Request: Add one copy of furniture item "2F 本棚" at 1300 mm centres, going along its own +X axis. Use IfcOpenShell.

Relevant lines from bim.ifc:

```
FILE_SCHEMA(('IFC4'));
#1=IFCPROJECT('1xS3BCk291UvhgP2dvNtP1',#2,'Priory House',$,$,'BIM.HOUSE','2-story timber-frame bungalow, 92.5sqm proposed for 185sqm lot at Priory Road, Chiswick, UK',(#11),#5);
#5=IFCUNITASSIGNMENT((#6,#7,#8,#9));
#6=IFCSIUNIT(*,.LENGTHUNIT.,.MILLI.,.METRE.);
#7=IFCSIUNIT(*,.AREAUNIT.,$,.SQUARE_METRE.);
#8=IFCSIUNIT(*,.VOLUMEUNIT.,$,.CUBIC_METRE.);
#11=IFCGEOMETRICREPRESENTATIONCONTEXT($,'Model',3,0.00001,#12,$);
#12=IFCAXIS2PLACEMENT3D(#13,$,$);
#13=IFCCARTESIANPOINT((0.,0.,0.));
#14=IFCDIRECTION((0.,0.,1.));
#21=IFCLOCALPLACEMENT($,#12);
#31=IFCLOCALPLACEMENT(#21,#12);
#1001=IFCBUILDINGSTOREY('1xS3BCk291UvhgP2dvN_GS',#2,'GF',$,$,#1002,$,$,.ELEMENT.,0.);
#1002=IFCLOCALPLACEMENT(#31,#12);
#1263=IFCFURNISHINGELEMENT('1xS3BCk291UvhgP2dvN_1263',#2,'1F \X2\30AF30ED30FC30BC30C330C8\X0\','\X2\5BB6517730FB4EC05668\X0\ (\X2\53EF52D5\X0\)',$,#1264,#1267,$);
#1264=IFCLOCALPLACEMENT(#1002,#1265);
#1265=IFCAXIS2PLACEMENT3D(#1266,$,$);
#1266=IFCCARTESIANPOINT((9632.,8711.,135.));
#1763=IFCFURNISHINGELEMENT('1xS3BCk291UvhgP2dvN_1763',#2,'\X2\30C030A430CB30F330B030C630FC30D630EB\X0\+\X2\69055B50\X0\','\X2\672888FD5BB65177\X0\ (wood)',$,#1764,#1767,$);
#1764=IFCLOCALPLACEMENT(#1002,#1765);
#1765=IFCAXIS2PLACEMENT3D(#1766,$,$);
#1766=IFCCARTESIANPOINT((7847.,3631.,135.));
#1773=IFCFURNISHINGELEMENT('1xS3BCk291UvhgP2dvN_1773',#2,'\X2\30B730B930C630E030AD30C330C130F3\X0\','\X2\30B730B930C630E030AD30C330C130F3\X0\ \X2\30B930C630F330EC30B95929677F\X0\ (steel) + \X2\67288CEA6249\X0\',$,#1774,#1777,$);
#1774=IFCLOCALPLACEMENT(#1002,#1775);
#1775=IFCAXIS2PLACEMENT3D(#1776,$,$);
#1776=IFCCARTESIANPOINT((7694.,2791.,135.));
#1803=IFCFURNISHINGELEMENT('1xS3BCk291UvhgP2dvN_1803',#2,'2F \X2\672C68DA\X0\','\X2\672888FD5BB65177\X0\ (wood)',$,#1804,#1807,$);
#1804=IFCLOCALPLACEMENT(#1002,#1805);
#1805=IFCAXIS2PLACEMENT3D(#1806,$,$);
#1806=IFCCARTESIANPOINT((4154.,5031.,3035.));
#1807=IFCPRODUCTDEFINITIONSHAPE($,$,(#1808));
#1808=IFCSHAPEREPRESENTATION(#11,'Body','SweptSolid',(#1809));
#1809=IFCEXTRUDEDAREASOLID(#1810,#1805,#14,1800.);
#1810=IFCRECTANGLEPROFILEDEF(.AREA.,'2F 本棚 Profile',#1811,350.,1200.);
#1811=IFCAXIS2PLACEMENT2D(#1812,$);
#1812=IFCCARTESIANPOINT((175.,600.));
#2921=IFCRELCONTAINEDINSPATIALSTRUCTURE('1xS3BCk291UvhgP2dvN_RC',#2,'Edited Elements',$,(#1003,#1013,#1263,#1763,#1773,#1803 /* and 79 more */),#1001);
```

```python
import ifcopenshell
import ifcopenshell.api.geometry
import ifcopenshell.api.root
import ifcopenshell.util.element
import ifcopenshell.util.placement
import ifcopenshell.util.unit

model = ifcopenshell.open("bim.ifc")
unit_scale = ifcopenshell.util.unit.calculate_unit_scale(model)


def reuse_history(source, copy):
    """copy_class also copies each property set's owner history, people and application; keep the originals."""
    for rel in copy.IsDefinedBy:
        if rel.is_a("IfcRelDefinesByProperties") and (history := rel.RelatingPropertyDefinition.OwnerHistory):
            rel.RelatingPropertyDefinition.OwnerHistory = source.OwnerHistory
            ifcopenshell.util.element.remove_deep2(model, history)


source = model.by_guid("1xS3BCk291UvhgP2dvN_1803")
base = ifcopenshell.util.placement.get_local_placement(source.ObjectPlacement)
step = base[:3, 0] * 1.3 / unit_scale

for i in range(1, 2):
    copy = ifcopenshell.api.root.copy_class(model, product=source)
    copy.Representation = ifcopenshell.util.element.copy_deep(
        model, source.Representation, exclude=["IfcGeometricRepresentationContext", "IfcRepresentationMap"]
    )
    reuse_history(source, copy)
    matrix = base.copy()
    matrix[:3, 3] += i * step
    print("added at", matrix[:3, 3].round(3) + 0.0)
    ifcopenshell.api.geometry.edit_object_placement(model, product=copy, matrix=matrix, is_si=False)

model.write("bim_rev.ifc")
```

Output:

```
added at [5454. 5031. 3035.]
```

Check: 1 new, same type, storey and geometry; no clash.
